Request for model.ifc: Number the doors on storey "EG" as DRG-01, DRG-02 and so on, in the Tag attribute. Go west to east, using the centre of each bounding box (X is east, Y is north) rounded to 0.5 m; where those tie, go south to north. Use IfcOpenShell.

First a look at what the model holds.

```python
import ifcopenshell
import ifcopenshell.util.element
import ifcopenshell.util.placement

model = ifcopenshell.open("model.ifc")
print(model.schema)
storey = next(s for s in model.by_type("IfcBuildingStorey") if s.Name == "EG")
doors = [e for e in ifcopenshell.util.element.get_decomposition(storey) if e.is_a("IfcDoor")]
for e in sorted(doors, key=lambda e: e.id()):
    origin = ifcopenshell.util.placement.get_local_placement(e.ObjectPlacement)[:3, 3]
    print(e.id(), e.Tag, e.Name, origin.round(2) + 0.0, sep=" | ")
```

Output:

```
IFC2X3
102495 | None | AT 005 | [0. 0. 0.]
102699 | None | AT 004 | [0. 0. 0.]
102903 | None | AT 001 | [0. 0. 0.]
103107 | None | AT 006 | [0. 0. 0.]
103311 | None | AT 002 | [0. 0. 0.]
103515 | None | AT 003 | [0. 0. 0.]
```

```python
import ifcopenshell
import ifcopenshell.geom
import ifcopenshell.util.element
import ifcopenshell.util.shape

model = ifcopenshell.open("model.ifc")
settings = ifcopenshell.geom.settings()
settings.set("use-world-coords", True)


def centre(element):
    shape = ifcopenshell.geom.create_shape(settings, element)
    return ifcopenshell.util.shape.get_bbox_centroid(shape.geometry)


storey = next(s for s in model.by_type("IfcBuildingStorey") if s.Name == "EG")
doors = [e for e in ifcopenshell.util.element.get_decomposition(storey) if e.is_a("IfcDoor")]

# Insertion points can sit at a corner or the storey origin, so sort by the geometry (in metres).
centres = {e: centre(e) for e in doors}
doors.sort(key=lambda e: (round(centres[e][0] / 0.5), centres[e][1]))

for i, e in enumerate(doors, start=1):
    number = f"DRG-{i:02d}"
    e.Tag = number
    print(e.id(), number)

model.write("model-out.ifc")
```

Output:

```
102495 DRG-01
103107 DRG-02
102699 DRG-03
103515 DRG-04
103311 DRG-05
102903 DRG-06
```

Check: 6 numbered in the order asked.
